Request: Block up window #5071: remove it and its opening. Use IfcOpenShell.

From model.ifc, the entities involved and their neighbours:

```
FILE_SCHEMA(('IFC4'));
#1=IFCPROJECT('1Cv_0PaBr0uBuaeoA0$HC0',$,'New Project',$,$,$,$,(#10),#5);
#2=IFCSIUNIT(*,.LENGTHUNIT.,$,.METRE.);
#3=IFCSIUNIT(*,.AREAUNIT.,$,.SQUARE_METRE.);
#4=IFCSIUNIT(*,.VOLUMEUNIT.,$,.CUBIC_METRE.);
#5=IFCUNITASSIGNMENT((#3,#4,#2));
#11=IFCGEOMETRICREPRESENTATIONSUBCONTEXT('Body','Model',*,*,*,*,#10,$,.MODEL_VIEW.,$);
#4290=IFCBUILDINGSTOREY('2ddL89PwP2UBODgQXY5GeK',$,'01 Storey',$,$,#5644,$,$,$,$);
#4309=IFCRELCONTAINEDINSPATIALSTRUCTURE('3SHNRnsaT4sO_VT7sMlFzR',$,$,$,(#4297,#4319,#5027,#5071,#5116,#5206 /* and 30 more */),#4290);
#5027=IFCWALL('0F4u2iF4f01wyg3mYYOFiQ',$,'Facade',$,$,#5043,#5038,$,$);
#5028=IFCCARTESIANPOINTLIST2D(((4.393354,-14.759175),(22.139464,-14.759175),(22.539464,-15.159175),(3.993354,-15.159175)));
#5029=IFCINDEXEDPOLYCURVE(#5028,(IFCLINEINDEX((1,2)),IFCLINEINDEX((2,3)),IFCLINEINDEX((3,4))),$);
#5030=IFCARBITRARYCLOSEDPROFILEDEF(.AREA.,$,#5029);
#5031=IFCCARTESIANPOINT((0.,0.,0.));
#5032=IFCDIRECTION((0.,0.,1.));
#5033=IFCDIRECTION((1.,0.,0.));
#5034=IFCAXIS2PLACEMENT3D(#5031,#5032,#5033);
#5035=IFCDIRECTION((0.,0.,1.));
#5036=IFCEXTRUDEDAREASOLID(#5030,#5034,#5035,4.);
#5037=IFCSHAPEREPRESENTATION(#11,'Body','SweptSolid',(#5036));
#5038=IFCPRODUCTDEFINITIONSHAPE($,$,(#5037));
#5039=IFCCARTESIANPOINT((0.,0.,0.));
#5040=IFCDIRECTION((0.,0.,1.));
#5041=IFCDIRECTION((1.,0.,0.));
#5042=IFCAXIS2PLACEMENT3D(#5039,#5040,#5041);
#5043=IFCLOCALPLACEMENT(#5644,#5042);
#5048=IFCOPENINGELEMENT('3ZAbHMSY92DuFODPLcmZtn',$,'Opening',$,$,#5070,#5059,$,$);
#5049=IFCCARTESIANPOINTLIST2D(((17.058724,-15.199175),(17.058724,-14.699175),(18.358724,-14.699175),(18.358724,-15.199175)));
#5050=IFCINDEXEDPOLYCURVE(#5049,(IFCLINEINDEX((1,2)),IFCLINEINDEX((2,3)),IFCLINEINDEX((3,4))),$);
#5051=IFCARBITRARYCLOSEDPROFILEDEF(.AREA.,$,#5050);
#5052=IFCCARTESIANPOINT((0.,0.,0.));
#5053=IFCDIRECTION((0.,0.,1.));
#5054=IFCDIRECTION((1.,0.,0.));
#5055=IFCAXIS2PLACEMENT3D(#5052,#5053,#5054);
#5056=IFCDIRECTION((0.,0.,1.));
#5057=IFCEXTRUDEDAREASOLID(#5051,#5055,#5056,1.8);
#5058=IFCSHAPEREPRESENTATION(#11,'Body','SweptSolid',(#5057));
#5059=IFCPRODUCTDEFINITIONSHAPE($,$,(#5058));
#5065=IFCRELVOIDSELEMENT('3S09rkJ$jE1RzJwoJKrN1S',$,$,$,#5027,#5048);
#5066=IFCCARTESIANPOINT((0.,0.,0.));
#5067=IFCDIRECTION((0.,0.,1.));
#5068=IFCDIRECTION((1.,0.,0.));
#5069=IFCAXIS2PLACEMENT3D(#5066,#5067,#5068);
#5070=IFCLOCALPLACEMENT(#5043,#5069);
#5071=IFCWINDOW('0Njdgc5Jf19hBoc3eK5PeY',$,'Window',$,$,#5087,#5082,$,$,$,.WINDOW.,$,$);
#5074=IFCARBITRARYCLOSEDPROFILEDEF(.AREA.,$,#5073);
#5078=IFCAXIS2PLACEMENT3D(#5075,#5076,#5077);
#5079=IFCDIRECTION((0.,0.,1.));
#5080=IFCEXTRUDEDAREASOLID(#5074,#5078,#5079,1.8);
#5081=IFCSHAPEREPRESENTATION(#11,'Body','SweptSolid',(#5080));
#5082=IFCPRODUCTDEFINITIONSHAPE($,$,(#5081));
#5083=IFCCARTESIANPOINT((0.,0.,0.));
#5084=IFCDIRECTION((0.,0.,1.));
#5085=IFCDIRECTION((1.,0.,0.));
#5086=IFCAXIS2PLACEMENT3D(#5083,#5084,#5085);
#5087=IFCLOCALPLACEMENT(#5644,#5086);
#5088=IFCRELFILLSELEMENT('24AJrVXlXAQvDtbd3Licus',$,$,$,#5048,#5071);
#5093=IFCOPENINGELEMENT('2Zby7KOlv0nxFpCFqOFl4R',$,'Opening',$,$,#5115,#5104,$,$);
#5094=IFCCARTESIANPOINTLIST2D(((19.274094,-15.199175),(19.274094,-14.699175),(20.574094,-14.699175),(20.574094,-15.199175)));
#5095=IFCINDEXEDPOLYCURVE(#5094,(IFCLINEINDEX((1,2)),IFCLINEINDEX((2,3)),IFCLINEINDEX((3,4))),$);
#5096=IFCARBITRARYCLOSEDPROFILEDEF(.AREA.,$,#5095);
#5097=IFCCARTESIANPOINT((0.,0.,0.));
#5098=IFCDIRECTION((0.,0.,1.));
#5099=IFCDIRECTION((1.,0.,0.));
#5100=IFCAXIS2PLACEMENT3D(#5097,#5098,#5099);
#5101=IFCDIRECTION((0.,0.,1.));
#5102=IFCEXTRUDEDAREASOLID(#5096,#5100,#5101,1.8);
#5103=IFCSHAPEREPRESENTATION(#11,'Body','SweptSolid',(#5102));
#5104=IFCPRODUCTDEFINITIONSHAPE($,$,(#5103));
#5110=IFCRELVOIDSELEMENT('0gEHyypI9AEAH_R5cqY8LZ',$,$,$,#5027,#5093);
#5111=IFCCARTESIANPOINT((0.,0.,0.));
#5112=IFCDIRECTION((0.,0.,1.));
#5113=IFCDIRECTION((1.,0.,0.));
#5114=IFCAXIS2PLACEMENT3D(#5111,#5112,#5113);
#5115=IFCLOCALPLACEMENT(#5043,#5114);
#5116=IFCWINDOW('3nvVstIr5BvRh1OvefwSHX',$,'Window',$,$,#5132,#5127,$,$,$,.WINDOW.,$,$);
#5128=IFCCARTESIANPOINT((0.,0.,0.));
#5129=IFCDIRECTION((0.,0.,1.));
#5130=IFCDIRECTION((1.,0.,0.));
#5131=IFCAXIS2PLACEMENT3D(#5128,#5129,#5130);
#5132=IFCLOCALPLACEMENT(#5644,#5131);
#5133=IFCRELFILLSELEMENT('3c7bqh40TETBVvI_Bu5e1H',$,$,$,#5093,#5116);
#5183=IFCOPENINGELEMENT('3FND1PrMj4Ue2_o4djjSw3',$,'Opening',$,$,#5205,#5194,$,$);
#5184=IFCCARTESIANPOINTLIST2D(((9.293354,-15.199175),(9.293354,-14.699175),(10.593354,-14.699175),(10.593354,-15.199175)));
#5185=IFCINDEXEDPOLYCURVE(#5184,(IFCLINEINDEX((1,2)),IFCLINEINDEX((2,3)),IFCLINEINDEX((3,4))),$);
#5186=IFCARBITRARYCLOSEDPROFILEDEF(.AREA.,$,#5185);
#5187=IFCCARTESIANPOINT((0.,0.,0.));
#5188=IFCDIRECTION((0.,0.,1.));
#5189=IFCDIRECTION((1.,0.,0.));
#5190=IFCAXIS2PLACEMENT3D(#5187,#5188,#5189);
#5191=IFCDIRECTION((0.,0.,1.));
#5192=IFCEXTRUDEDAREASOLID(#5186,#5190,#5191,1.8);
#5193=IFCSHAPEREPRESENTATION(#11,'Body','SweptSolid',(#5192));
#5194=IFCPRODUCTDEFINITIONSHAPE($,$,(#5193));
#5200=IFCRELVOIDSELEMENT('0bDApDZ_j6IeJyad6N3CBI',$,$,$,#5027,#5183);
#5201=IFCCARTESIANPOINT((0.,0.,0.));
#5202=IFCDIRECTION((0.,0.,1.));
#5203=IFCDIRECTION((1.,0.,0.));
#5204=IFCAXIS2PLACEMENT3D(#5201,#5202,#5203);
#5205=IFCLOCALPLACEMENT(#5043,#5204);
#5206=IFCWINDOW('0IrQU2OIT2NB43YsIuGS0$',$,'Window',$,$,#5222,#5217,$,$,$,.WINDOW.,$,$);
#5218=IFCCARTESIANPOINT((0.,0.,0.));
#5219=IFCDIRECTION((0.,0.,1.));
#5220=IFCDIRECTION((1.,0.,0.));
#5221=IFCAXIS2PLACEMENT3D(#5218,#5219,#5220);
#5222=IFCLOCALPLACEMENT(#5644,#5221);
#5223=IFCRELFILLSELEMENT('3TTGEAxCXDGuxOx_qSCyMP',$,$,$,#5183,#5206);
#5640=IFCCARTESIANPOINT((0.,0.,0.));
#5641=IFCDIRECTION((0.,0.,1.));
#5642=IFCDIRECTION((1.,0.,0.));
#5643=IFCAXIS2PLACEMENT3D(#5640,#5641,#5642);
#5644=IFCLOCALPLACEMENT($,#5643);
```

```python
import ifcopenshell
import ifcopenshell.api.feature
import ifcopenshell.api.root
import ifcopenshell.geom
import ifcopenshell.util.shape

model = ifcopenshell.open("model.ifc")
settings = ifcopenshell.geom.settings()


def volume(element):
    """Net volume in cubic metres, openings subtracted."""
    shape = ifcopenshell.geom.create_shape(settings, element)
    return ifcopenshell.util.shape.get_volume(shape.geometry)


window = model.by_id(5071)
opening = window.FillsVoids[0].RelatingOpeningElement
wall = opening.VoidsElements[0].RelatingBuildingElement
before = volume(wall)

ifcopenshell.api.root.remove_product(model, product=window)
ifcopenshell.api.feature.remove_feature(model, feature=opening)

after = volume(wall)

print(f"wall volume {before:.3f} -> {after:.3f} m3")

model.write("model-out.ifc")
```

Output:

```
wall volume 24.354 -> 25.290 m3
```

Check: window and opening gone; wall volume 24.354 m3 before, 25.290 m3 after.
